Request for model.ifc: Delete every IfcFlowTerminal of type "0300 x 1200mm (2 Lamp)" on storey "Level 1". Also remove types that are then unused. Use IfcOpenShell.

First a look at what the model holds.

```python
import ifcopenshell
import ifcopenshell.util.element

model = ifcopenshell.open("model.ifc")
print(model.schema)
storey = next(s for s in model.by_type("IfcBuildingStorey") if s.Name == "Level 1")
terminals = [e for e in ifcopenshell.util.element.get_decomposition(storey) if e.is_a("IfcFlowTerminal")]
seen = {}
for e in terminals:
    element_type = ifcopenshell.util.element.get_type(e)
    name = element_type.Name if element_type not in (None, e) else None
    seen[name] = seen.get(name, 0) + 1
for name, count in sorted(seen.items(), key=str):
    print(count, "x", name)
```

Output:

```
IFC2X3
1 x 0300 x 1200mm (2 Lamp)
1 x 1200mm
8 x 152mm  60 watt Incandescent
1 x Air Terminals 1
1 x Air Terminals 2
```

```python
import ifcopenshell
import ifcopenshell.api.root
import ifcopenshell.util.element

model = ifcopenshell.open("model.ifc")

storey = next(s for s in model.by_type("IfcBuildingStorey") if s.Name == "Level 1")
terminals = [e for e in ifcopenshell.util.element.get_decomposition(storey) if e.is_a("IfcFlowTerminal")]
targets = [e for e in terminals if (t := ifcopenshell.util.element.get_type(e)) not in (None, e) and t.Name == "0300 x 1200mm (2 Lamp)"]
types = {ifcopenshell.util.element.get_type(e) for e in targets} - {None, *targets}

for e in targets:
    ifcopenshell.api.root.remove_product(model, product=e)
print(len(targets), "removed")

unused = [t for t in types if not ifcopenshell.util.element.get_types(t)]
for t in unused:
    ifcopenshell.api.root.remove_product(model, product=t)
print(len(unused), "unused types removed")

model.write("model-out.ifc")
```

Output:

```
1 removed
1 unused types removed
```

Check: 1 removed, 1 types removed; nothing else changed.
